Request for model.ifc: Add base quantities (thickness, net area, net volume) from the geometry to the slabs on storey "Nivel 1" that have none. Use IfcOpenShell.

First a look at what the model holds.

```python
import ifcopenshell
import ifcopenshell.util.element
import ifcopenshell.util.unit

model = ifcopenshell.open("model.ifc")
print(model.schema)
for unit_type in ("LENGTHUNIT", "AREAUNIT", "VOLUMEUNIT"):
    print(unit_type, ifcopenshell.util.unit.calculate_unit_scale(model, unit_type))
storey = next(s for s in model.by_type("IfcBuildingStorey") if s.Name == "Nivel 1")
slabs = [e for e in ifcopenshell.util.element.get_decomposition(storey) if e.is_a("IfcSlab")]
for e in sorted(slabs, key=lambda e: e.id()):
    print(e.id(), e.is_a(), e.Name, list(ifcopenshell.util.element.get_psets(e, qtos_only=True)), sep=" | ")
```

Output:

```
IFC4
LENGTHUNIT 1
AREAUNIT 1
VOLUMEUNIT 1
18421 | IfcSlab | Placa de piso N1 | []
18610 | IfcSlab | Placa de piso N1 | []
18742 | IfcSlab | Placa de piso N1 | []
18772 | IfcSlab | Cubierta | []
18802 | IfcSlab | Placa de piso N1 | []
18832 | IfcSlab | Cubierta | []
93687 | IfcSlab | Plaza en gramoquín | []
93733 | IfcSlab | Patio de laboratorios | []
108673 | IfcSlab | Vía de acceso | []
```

```python
import ifcopenshell
import ifcopenshell.api.pset
import ifcopenshell.geom
import ifcopenshell.util.element
import ifcopenshell.util.shape
import ifcopenshell.util.unit

model = ifcopenshell.open("model.ifc")
unit_scale = ifcopenshell.util.unit.calculate_unit_scale(model)
area_scale = ifcopenshell.util.unit.calculate_unit_scale(model, "AREAUNIT")
volume_scale = ifcopenshell.util.unit.calculate_unit_scale(model, "VOLUMEUNIT")
settings = ifcopenshell.geom.settings()

storey = next(s for s in model.by_type("IfcBuildingStorey") if s.Name == "Nivel 1")
slabs = [e for e in ifcopenshell.util.element.get_decomposition(storey) if e.is_a("IfcSlab")]

for e in sorted(slabs, key=lambda e: e.id()):
    if ifcopenshell.util.element.get_psets(e, qtos_only=True, should_inherit=False):
        continue
    # Geometry comes back in metres, in the element's own axes.
    shape = ifcopenshell.geom.create_shape(settings, e)
    values = {
        "Width": ifcopenshell.util.shape.get_z(shape.geometry) / unit_scale,
        "NetArea": ifcopenshell.util.shape.get_footprint_area(shape.geometry) / area_scale,
        "NetVolume": ifcopenshell.util.shape.get_volume(shape.geometry) / volume_scale,
    }
    qto = ifcopenshell.api.pset.add_qto(model, product=e, name="Qto_SlabBaseQuantities")
    ifcopenshell.api.pset.edit_qto(model, qto=qto, properties=values)
    print(e.id(), {k: round(v, 3) for k, v in values.items()})

model.write("model-out.ifc")
```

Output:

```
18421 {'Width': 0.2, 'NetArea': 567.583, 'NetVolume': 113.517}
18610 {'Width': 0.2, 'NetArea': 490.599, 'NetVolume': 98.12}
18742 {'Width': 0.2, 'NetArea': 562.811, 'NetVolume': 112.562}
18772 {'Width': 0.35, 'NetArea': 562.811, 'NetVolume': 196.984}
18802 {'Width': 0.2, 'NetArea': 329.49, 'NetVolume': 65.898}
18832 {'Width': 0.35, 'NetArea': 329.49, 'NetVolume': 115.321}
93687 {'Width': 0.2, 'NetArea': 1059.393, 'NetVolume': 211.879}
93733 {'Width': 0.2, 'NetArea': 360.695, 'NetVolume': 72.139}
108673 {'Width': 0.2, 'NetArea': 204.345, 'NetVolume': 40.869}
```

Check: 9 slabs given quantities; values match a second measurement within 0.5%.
